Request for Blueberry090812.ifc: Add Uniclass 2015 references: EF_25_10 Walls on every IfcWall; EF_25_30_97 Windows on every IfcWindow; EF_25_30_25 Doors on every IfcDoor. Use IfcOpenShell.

First a look at what the model holds.

```python
import ifcopenshell

model = ifcopenshell.open("Blueberry090812.ifc")
print(model.schema)
print("classifications:", [c.Name for c in model.by_type("IfcClassification")])
for ifc_class in ("IfcDoor", "IfcRoof", "IfcStair", "IfcWall", "IfcWindow"):
    print(ifc_class, len(model.by_type(ifc_class)))
```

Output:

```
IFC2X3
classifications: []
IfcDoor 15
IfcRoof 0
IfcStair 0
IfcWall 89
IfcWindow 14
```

```python
import ifcopenshell
import ifcopenshell.api.classification

model = ifcopenshell.open("Blueberry090812.ifc")

# IFC2X3 requires Source and Edition and has no link from the project to the system.
system = model.create_entity("IfcClassification", Source="NBS", Edition="2015", Name="Uniclass 2015")

codes = {
    "IfcWall": ("EF_25_10", "Walls"),
    "IfcWindow": ("EF_25_30_97", "Windows"),
    "IfcDoor": ("EF_25_30_25", "Doors"),
}
for ifc_class, (code, name) in codes.items():
    products = model.by_type(ifc_class)
    ifcopenshell.api.classification.add_reference(
        model, products=products, classification=system, identification=code, name=name
    )
    print(code, len(products))

model.write("Blueberry090812_updated.ifc")
```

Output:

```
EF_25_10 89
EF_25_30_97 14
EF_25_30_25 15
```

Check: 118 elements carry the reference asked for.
